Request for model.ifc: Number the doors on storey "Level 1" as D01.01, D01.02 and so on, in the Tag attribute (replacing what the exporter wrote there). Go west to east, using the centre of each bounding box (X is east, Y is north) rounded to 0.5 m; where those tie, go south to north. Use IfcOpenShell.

First a look at what the model holds.

```python
import ifcopenshell
import ifcopenshell.util.element
import ifcopenshell.util.placement

model = ifcopenshell.open("model.ifc")
print(model.schema)
storey = next(s for s in model.by_type("IfcBuildingStorey") if s.Name == "Level 1")
doors = [e for e in ifcopenshell.util.element.get_decomposition(storey) if e.is_a("IfcDoor")]
for e in sorted(doors, key=lambda e: e.id()):
    origin = ifcopenshell.util.placement.get_local_placement(e.ObjectPlacement)[:3, 3]
    print(e.id(), e.Tag, e.Name, origin.round(2) + 0.0, sep=" | ")
```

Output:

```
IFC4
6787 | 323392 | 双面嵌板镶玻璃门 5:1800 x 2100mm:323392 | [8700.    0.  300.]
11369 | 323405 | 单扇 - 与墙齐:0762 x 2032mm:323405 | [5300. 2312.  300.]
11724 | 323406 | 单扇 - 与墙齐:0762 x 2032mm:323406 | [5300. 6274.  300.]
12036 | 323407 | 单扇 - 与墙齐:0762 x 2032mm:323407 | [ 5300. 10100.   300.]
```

```python
import ifcopenshell
import ifcopenshell.geom
import ifcopenshell.util.element
import ifcopenshell.util.shape

model = ifcopenshell.open("model.ifc")
settings = ifcopenshell.geom.settings()
settings.set("use-world-coords", True)


def centre(element):
    shape = ifcopenshell.geom.create_shape(settings, element)
    return ifcopenshell.util.shape.get_bbox_centroid(shape.geometry)


storey = next(s for s in model.by_type("IfcBuildingStorey") if s.Name == "Level 1")
doors = [e for e in ifcopenshell.util.element.get_decomposition(storey) if e.is_a("IfcDoor")]

# Insertion points can sit at a corner or the storey origin, so sort by the geometry (in metres).
centres = {e: centre(e) for e in doors}
doors.sort(key=lambda e: (round(centres[e][0] / 0.5), centres[e][1]))

for i, e in enumerate(doors, start=1):
    number = f"D01.{i:02d}"
    e.Tag = number
    print(e.id(), number)

model.write("model_edited.ifc")
```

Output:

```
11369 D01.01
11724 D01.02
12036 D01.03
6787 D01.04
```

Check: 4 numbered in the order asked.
